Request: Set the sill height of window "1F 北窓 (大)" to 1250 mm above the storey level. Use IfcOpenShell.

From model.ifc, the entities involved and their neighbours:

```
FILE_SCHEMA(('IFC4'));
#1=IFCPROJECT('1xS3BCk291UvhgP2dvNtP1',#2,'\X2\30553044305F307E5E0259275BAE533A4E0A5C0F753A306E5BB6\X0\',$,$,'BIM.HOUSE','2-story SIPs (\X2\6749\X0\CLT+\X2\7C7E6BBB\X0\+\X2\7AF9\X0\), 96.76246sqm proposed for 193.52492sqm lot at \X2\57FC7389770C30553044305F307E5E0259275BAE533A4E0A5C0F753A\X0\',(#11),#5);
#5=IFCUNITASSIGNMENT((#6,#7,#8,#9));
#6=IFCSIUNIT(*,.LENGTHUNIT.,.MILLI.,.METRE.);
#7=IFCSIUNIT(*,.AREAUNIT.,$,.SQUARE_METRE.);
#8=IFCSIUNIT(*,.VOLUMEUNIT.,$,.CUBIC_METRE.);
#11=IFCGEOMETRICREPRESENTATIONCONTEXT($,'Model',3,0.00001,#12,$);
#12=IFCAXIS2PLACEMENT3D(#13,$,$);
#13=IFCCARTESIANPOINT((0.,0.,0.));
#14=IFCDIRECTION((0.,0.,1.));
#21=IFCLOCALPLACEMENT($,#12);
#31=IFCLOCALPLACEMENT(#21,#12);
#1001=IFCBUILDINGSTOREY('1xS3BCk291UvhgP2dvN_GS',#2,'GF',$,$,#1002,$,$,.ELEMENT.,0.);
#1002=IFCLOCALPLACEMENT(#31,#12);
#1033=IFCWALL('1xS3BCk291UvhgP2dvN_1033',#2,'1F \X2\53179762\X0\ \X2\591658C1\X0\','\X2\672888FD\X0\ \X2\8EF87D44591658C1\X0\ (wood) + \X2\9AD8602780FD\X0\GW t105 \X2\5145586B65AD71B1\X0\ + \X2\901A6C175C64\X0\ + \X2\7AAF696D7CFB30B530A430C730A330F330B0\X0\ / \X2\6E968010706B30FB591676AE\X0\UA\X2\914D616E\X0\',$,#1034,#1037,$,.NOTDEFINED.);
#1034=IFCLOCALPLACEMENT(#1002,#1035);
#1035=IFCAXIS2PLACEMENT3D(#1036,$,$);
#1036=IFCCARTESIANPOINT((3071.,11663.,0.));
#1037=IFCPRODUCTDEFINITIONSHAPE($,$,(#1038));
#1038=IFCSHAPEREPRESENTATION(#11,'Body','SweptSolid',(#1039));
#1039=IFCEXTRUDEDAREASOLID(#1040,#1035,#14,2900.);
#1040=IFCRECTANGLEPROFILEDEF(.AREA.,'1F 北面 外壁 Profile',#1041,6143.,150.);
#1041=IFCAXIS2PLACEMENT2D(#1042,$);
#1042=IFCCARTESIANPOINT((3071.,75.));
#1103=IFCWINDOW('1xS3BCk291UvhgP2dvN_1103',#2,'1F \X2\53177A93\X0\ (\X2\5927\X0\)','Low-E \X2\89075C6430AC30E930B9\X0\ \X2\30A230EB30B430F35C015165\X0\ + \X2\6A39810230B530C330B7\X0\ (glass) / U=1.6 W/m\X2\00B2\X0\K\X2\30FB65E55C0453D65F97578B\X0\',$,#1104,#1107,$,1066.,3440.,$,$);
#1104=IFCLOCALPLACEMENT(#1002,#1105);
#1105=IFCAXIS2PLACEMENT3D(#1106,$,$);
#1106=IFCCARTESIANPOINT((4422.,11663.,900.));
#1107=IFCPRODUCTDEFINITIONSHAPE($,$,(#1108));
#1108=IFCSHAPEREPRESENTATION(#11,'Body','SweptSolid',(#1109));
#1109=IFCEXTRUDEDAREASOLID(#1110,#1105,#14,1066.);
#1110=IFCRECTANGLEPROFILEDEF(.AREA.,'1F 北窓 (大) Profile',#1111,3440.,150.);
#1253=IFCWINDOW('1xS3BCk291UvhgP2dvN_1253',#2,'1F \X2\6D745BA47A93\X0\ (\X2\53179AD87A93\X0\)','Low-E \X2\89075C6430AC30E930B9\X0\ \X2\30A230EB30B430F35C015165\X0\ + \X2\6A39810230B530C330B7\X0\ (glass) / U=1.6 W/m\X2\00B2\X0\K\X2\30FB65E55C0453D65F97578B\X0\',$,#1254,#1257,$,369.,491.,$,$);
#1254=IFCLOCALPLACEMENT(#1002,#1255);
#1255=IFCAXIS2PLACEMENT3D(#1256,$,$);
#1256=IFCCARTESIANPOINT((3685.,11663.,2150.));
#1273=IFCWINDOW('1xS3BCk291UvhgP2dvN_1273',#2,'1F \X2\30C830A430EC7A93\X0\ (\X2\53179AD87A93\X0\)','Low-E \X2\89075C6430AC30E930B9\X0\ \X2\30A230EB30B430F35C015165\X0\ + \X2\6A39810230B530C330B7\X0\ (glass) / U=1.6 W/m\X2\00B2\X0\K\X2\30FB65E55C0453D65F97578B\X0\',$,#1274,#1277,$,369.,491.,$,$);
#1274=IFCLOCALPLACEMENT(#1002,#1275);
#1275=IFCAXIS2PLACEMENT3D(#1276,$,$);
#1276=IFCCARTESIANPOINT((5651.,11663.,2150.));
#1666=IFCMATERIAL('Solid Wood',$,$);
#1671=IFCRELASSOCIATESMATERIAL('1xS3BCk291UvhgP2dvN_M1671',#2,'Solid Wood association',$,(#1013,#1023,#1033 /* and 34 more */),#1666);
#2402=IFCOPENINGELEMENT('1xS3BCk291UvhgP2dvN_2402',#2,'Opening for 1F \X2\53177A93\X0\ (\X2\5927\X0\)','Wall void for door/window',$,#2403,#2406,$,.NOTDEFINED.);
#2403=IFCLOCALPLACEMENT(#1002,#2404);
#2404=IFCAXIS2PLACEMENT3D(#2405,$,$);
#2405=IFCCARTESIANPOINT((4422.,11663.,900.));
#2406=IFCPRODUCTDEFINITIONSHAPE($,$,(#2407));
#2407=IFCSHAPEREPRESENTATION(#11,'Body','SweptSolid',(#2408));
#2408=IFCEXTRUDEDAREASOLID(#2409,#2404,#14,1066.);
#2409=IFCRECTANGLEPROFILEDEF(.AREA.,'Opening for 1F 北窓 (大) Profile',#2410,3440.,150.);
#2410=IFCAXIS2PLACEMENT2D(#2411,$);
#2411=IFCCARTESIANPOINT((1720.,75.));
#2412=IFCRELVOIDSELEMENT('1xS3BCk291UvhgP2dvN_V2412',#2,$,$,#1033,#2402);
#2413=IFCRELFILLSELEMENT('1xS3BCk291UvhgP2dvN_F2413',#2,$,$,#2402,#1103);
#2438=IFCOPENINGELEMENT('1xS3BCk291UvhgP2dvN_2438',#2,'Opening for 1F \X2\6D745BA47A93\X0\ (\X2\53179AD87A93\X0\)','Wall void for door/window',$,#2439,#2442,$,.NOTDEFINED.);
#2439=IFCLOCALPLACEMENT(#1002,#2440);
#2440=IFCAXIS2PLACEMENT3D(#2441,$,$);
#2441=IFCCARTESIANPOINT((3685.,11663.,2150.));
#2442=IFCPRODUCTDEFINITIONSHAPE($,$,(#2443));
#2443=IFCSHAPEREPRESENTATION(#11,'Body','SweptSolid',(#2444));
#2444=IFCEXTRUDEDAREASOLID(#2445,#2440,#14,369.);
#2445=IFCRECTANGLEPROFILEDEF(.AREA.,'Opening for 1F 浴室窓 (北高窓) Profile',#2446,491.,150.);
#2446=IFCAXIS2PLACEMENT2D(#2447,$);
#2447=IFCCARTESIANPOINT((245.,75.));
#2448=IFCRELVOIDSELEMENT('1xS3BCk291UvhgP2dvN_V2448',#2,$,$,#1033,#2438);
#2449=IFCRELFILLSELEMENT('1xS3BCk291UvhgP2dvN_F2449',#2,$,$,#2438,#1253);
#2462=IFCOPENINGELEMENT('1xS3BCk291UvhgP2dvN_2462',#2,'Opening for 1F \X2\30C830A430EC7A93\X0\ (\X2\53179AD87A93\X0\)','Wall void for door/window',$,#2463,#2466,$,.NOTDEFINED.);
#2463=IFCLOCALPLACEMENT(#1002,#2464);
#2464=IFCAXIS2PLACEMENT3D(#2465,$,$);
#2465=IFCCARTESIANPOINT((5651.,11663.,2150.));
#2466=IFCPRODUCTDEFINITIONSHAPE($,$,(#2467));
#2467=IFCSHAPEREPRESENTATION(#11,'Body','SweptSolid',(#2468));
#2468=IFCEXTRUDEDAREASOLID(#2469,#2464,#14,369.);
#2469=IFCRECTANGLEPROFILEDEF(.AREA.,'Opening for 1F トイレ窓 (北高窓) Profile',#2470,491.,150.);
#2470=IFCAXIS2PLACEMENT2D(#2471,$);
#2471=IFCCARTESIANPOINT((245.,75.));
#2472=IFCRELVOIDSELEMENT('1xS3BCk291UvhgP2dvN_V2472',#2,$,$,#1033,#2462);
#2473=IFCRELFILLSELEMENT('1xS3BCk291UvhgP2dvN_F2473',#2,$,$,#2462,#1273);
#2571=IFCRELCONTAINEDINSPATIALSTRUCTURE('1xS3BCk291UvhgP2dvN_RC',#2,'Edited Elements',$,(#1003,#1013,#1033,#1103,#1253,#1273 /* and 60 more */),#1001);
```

```python
import numpy as np
import ifcopenshell
import ifcopenshell.api.geometry
import ifcopenshell.geom
import ifcopenshell.util.element
import ifcopenshell.util.placement
import ifcopenshell.util.shape
import ifcopenshell.util.unit

model = ifcopenshell.open("model.ifc")
unit_scale = ifcopenshell.util.unit.calculate_unit_scale(model)

window = model.by_id(1103)
opening = window.FillsVoids[0].RelatingOpeningElement
storey = ifcopenshell.util.element.get_container(window, ifc_class="IfcBuildingStorey")
level = ifcopenshell.util.placement.get_local_placement(storey.ObjectPlacement)[2, 3]

# The opening's origin need not be at the sill, so measure its lowest point.
shape = ifcopenshell.geom.create_shape(ifcopenshell.geom.settings(), opening)
bottom = ifcopenshell.util.shape.get_shape_bottom_elevation(shape, shape.geometry) / unit_scale
dz = level + 1250.0 - bottom

shift = np.array([0.0, 0.0, dz])
# The window is not placed relative to its opening, so move both.
for product in (opening, window):
    matrix = ifcopenshell.util.placement.get_local_placement(product.ObjectPlacement)
    matrix[:3, 3] += shift
    ifcopenshell.api.geometry.edit_object_placement(model, product=product, matrix=matrix, is_si=False)

print(f"moved by {dz * unit_scale:+.3f} m")

model.write("model_rev.ifc")
```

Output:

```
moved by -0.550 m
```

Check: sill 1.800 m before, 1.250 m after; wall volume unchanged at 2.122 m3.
